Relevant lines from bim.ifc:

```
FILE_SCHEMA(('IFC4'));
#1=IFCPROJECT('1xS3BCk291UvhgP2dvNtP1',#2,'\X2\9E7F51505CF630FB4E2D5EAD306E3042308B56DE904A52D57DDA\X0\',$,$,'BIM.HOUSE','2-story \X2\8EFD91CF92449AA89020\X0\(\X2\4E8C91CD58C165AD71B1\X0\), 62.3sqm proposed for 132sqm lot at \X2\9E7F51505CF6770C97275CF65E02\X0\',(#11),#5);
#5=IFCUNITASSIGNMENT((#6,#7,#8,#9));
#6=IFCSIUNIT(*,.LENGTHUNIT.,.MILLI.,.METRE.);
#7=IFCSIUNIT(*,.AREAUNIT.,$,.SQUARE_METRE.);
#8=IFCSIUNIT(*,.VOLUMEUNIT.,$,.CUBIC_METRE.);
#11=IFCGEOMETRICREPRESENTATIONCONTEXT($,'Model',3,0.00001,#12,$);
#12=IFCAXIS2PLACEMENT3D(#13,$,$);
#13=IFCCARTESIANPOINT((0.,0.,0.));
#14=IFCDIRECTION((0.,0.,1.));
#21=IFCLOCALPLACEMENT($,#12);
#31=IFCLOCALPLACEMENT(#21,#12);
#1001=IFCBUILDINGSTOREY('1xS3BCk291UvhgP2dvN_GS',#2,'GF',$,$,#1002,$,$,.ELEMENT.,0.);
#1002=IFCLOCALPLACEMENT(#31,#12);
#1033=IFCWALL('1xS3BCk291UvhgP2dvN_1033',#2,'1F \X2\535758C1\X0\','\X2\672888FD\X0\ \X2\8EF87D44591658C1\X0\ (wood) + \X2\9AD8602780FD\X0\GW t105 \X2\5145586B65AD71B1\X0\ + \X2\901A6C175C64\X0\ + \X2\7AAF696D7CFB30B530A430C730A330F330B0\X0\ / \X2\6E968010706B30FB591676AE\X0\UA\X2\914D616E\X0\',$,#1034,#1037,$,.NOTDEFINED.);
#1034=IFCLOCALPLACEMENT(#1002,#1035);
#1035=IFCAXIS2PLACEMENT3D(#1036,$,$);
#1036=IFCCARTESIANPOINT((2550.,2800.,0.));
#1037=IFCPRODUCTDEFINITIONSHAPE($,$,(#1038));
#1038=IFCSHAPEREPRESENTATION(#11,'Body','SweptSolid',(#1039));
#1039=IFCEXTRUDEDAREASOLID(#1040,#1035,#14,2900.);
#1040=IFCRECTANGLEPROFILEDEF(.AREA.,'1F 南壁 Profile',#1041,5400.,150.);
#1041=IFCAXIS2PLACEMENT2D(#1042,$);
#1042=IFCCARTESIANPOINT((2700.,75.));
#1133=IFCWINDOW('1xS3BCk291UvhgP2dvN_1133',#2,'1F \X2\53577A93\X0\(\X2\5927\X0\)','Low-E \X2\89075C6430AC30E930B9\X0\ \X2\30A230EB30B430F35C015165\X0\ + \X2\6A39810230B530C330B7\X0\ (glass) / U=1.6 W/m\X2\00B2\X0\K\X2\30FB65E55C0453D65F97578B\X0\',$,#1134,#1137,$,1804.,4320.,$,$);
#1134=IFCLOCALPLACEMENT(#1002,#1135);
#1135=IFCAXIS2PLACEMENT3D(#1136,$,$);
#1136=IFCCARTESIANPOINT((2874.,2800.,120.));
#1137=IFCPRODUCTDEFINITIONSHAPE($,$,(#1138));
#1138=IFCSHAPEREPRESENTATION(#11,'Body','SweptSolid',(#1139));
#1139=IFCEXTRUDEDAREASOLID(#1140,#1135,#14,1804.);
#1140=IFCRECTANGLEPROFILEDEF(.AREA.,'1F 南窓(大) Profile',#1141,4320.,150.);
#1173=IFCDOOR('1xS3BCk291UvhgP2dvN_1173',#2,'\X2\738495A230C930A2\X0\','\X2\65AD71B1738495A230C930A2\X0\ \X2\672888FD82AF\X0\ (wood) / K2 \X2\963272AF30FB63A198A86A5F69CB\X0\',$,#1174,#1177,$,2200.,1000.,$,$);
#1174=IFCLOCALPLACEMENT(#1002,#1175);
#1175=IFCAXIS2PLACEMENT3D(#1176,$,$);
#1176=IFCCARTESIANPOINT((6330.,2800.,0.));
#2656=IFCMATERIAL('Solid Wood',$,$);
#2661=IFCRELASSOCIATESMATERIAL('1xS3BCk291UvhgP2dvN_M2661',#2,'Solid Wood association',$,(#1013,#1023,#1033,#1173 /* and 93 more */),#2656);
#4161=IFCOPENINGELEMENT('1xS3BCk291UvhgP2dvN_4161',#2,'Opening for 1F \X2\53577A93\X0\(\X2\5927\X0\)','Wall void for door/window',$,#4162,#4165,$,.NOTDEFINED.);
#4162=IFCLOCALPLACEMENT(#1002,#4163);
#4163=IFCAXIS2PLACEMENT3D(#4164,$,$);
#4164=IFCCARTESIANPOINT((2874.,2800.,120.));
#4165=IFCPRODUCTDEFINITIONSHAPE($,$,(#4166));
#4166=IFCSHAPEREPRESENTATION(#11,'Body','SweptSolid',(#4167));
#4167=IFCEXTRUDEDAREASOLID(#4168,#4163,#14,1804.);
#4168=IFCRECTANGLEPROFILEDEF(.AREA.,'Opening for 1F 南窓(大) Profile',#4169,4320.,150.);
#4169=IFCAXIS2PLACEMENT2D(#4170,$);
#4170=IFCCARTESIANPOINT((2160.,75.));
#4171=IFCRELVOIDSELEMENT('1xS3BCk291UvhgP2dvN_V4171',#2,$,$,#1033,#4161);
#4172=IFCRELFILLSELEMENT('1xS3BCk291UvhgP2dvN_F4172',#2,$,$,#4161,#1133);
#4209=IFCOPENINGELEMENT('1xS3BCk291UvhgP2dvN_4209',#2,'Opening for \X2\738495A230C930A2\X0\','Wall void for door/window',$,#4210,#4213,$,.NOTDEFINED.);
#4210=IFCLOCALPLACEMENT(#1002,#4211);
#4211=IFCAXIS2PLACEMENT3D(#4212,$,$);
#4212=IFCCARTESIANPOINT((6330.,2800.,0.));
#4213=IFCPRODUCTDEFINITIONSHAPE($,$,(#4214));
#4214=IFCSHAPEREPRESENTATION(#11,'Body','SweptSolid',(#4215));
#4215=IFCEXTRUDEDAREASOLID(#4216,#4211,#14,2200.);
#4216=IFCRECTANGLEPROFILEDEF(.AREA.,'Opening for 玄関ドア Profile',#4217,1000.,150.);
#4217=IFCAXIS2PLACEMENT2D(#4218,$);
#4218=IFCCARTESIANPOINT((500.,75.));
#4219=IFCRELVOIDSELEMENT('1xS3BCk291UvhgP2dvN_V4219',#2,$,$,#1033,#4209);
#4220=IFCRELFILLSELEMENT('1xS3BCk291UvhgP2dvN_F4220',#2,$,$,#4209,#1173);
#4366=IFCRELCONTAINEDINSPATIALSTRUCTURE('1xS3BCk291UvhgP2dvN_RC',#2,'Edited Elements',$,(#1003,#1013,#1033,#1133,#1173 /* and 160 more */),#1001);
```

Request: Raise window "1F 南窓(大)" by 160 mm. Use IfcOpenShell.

```python
import numpy as np
import ifcopenshell
import ifcopenshell.api.geometry
import ifcopenshell.util.placement
import ifcopenshell.util.unit

model = ifcopenshell.open("bim.ifc")
unit_scale = ifcopenshell.util.unit.calculate_unit_scale(model)

window = model.by_guid("1xS3BCk291UvhgP2dvN_1133")
opening = window.FillsVoids[0].RelatingOpeningElement
dz = 160.0

shift = np.array([0.0, 0.0, dz])
# The window is not placed relative to its opening, so move both.
for product in (opening, window):
    matrix = ifcopenshell.util.placement.get_local_placement(product.ObjectPlacement)
    matrix[:3, 3] += shift
    ifcopenshell.api.geometry.edit_object_placement(model, product=product, matrix=matrix, is_si=False)

print(f"moved by {dz * unit_scale:+.3f} m")

model.write("bim_rev.ifc")
```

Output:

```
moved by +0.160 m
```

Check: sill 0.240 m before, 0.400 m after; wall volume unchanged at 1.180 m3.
